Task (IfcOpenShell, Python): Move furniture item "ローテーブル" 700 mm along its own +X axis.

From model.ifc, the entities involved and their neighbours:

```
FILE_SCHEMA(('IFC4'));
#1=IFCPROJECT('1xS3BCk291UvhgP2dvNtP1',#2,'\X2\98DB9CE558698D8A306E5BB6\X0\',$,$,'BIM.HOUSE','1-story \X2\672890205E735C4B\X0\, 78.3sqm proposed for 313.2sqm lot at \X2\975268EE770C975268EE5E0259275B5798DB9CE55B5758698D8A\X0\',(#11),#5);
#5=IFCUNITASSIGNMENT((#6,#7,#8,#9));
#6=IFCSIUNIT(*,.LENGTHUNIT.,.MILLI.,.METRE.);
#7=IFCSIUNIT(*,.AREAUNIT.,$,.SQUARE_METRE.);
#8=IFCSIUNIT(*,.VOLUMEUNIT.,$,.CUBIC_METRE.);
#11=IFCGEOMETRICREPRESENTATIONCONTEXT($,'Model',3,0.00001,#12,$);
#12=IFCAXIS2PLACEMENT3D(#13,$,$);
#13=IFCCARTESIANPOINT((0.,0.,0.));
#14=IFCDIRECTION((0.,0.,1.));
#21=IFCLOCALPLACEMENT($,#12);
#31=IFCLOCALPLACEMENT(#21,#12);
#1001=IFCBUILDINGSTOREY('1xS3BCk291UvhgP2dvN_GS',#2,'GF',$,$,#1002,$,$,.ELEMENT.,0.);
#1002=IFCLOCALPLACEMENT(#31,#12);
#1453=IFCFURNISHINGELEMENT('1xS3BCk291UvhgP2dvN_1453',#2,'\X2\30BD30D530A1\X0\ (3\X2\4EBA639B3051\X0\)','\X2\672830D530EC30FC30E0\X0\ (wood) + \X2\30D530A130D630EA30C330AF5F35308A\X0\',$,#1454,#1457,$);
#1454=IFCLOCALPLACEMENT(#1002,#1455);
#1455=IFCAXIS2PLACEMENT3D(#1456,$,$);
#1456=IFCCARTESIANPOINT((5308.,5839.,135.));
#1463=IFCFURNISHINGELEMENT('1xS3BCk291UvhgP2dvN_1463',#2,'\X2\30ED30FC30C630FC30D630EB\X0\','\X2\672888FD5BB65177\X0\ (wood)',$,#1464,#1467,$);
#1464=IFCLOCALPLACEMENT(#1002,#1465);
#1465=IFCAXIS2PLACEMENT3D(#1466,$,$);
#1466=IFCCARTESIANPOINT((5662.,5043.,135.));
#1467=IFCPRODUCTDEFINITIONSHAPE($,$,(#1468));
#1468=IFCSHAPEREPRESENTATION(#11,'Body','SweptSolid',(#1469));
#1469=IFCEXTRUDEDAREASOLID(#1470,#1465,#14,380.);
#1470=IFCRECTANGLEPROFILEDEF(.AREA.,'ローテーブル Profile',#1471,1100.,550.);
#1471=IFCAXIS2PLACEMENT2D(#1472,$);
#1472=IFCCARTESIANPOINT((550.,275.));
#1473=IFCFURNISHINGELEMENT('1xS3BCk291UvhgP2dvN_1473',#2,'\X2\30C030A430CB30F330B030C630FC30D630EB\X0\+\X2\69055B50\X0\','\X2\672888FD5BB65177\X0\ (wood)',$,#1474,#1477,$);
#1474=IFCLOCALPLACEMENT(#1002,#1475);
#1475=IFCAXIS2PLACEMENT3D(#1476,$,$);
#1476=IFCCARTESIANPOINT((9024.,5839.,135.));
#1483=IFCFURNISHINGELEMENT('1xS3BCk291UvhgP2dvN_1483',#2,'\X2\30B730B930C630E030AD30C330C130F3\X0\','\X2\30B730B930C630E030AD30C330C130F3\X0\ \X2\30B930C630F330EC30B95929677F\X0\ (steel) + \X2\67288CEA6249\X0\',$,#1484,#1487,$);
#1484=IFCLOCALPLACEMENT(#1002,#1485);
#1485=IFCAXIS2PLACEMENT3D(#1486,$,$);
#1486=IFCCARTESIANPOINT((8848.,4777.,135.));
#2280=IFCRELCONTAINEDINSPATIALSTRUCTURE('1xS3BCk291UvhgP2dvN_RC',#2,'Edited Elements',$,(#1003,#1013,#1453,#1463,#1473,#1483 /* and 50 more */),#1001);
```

```python
import ifcopenshell
import ifcopenshell.api.geometry
import ifcopenshell.util.placement

model = ifcopenshell.open("model.ifc")

item = model.by_guid("1xS3BCk291UvhgP2dvN_1463")
matrix = ifcopenshell.util.placement.get_local_placement(item.ObjectPlacement)
matrix[:3, 3] += matrix[:3, 0] * 700.0
ifcopenshell.api.geometry.edit_object_placement(model, product=item, matrix=matrix, is_si=False)

print(ifcopenshell.util.placement.get_local_placement(item.ObjectPlacement).round(3) + 0.0)

model.write("model_v2.ifc")
```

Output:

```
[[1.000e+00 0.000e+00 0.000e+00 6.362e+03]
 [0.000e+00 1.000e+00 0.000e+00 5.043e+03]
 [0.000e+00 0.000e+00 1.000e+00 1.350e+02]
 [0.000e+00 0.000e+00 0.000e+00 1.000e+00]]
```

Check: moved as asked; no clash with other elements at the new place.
